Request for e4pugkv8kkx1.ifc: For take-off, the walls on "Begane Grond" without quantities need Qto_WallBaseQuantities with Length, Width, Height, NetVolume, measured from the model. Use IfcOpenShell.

First a look at what the model holds.

```python
import ifcopenshell
import ifcopenshell.util.element
import ifcopenshell.util.unit

model = ifcopenshell.open("e4pugkv8kkx1.ifc")
print(model.schema)
for unit_type in ("LENGTHUNIT", "AREAUNIT", "VOLUMEUNIT"):
    print(unit_type, ifcopenshell.util.unit.calculate_unit_scale(model, unit_type))
storey = next(s for s in model.by_type("IfcBuildingStorey") if s.Name == "Begane Grond")
walls = [e for e in ifcopenshell.util.element.get_decomposition(storey) if e.is_a("IfcWall")]
for e in sorted(walls, key=lambda e: e.id()):
    print(e.id(), e.is_a(), e.Name, list(ifcopenshell.util.element.get_psets(e, qtos_only=True)), sep=" | ")
```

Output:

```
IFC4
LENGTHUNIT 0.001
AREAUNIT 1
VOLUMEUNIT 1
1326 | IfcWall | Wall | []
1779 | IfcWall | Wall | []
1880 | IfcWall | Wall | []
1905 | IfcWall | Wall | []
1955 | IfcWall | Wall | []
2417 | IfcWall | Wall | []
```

```python
import ifcopenshell
import ifcopenshell.api.pset
import ifcopenshell.geom
import ifcopenshell.util.element
import ifcopenshell.util.shape
import ifcopenshell.util.unit

model = ifcopenshell.open("e4pugkv8kkx1.ifc")
unit_scale = ifcopenshell.util.unit.calculate_unit_scale(model)
volume_scale = ifcopenshell.util.unit.calculate_unit_scale(model, "VOLUMEUNIT")
settings = ifcopenshell.geom.settings()

storey = next(s for s in model.by_type("IfcBuildingStorey") if s.Name == "Begane Grond")
walls = [e for e in ifcopenshell.util.element.get_decomposition(storey) if e.is_a("IfcWall")]

for e in sorted(walls, key=lambda e: e.id()):
    if ifcopenshell.util.element.get_psets(e, qtos_only=True, should_inherit=False):
        continue
    # Geometry comes back in metres, in the element's own axes.
    shape = ifcopenshell.geom.create_shape(settings, e)
    values = {
        "Length": ifcopenshell.util.shape.get_x(shape.geometry) / unit_scale,
        "Width": ifcopenshell.util.shape.get_y(shape.geometry) / unit_scale,
        "Height": ifcopenshell.util.shape.get_z(shape.geometry) / unit_scale,
        "NetVolume": ifcopenshell.util.shape.get_volume(shape.geometry) / volume_scale,
    }
    qto = ifcopenshell.api.pset.add_qto(model, product=e, name="Qto_WallBaseQuantities")
    ifcopenshell.api.pset.edit_qto(model, qto=qto, properties=values)
    print(e.id(), {k: round(v, 3) for k, v in values.items()})

model.write("e4pugkv8kkx1_updated.ifc")
```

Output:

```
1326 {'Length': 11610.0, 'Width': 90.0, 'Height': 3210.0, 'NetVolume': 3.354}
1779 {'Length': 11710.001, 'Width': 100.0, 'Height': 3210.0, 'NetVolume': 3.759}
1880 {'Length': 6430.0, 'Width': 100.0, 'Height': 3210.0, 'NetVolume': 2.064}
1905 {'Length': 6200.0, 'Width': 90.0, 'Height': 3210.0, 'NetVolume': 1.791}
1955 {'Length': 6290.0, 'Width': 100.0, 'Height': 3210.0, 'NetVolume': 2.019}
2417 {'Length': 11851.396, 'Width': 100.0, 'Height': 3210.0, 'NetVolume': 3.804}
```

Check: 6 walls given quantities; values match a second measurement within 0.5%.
